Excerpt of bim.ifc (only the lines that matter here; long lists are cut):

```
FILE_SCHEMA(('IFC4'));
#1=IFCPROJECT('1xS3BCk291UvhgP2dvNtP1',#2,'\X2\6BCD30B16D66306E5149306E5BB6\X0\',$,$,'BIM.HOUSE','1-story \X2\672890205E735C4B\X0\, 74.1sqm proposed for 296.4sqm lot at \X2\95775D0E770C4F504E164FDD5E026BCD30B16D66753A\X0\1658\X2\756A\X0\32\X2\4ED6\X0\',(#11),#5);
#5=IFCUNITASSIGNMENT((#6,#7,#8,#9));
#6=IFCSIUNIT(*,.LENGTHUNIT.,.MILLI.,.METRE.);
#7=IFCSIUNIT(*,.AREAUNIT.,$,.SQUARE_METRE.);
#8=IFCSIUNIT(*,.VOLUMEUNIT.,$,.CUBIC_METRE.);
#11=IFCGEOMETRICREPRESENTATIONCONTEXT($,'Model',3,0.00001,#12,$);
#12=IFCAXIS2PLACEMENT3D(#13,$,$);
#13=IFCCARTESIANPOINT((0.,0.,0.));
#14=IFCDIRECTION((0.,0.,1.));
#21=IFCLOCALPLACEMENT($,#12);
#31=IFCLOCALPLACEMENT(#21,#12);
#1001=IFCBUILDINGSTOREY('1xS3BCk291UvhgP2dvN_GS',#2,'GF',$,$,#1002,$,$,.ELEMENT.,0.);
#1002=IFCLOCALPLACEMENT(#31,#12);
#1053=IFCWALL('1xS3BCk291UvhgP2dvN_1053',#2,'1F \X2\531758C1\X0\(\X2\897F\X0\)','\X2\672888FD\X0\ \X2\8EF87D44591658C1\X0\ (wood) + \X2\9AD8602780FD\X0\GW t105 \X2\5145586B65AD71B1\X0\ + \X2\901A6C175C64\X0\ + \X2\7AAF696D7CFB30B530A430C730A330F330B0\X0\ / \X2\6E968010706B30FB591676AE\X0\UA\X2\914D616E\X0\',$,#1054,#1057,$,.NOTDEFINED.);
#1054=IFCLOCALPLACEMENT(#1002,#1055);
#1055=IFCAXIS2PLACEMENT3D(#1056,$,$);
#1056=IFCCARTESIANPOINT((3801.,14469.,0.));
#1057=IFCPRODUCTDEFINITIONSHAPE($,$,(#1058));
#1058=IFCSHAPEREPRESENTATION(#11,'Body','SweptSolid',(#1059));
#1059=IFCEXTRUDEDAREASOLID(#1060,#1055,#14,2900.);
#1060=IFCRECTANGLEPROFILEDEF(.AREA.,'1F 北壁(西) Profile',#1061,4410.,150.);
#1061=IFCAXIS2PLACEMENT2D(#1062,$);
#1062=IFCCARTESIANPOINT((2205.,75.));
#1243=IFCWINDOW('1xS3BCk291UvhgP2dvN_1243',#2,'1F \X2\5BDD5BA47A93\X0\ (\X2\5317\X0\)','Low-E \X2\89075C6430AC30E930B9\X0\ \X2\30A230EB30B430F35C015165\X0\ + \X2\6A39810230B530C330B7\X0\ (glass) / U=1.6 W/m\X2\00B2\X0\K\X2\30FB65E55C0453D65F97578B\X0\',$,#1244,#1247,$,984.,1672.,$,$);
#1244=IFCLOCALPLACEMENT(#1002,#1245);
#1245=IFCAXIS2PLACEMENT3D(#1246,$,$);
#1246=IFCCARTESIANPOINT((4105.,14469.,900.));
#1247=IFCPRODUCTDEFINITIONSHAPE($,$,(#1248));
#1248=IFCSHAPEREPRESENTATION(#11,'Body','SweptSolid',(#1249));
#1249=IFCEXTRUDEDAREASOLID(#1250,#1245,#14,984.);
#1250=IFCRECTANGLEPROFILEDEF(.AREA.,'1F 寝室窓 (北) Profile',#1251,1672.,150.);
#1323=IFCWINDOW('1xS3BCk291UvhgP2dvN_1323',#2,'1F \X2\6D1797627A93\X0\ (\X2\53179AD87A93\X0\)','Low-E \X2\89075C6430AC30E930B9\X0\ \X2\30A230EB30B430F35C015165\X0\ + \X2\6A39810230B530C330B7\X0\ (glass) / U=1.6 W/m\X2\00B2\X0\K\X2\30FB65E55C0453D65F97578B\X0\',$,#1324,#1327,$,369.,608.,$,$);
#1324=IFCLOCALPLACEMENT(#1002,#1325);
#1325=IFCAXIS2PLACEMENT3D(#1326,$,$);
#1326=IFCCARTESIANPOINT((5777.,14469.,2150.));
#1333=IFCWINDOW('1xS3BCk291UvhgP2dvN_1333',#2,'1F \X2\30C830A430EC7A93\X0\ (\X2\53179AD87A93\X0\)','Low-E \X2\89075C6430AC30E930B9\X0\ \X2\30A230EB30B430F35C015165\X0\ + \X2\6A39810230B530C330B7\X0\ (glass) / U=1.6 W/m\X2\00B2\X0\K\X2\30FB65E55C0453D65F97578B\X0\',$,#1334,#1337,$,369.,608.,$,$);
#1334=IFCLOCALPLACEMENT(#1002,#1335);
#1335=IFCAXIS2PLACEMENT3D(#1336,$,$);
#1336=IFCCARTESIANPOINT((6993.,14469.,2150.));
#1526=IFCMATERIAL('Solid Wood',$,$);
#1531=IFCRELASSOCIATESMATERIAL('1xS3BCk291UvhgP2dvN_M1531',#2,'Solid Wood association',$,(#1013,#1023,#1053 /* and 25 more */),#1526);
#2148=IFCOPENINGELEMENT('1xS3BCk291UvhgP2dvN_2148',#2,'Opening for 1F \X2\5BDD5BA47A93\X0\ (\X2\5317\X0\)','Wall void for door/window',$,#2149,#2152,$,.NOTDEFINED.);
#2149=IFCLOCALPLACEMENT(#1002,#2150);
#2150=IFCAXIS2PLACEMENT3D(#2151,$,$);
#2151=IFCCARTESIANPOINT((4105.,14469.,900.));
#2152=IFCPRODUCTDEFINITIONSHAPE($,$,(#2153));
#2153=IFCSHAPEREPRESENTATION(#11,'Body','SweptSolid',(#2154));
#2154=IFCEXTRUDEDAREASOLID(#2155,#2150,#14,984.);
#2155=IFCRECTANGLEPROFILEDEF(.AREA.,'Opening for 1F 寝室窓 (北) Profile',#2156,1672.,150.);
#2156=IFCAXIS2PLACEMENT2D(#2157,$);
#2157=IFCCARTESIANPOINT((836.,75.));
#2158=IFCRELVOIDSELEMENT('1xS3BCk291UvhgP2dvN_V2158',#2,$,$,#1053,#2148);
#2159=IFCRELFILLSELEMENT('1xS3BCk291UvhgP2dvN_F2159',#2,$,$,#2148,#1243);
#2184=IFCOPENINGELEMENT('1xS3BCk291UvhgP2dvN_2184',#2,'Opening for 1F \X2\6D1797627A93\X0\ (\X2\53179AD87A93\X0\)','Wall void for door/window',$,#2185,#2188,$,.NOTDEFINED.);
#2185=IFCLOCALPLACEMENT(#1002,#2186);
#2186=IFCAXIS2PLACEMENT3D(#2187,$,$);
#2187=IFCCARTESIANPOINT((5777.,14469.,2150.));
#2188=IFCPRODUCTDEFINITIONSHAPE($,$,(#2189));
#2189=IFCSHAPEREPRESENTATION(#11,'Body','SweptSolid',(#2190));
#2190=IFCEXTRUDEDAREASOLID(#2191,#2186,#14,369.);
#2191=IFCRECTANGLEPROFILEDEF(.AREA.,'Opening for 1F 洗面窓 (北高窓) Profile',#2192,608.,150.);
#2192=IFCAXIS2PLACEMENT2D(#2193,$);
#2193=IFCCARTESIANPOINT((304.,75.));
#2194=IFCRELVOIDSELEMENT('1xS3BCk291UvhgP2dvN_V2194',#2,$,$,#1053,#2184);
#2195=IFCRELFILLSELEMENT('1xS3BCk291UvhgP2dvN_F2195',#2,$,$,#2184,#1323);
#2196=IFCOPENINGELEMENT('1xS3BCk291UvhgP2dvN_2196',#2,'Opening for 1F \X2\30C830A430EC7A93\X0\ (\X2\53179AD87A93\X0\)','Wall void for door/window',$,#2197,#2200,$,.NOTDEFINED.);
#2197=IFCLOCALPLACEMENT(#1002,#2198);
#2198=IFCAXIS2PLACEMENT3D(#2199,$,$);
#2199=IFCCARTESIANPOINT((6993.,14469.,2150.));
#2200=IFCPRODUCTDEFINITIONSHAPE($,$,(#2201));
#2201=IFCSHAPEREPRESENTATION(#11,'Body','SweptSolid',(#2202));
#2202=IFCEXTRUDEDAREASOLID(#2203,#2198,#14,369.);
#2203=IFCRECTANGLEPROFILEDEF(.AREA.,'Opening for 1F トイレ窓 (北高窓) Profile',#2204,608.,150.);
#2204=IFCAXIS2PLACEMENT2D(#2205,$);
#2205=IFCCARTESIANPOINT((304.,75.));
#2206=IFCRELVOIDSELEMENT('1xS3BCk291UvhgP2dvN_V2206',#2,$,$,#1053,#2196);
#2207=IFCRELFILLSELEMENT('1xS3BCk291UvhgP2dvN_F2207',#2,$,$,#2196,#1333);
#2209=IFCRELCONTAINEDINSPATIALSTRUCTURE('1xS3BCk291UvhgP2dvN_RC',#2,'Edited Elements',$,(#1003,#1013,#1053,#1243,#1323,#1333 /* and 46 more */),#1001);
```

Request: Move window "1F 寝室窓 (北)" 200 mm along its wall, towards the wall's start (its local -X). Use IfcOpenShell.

```python
import ifcopenshell
import ifcopenshell.api.geometry
import ifcopenshell.util.placement
import ifcopenshell.util.unit

model = ifcopenshell.open("bim.ifc")
unit_scale = ifcopenshell.util.unit.calculate_unit_scale(model)

window = model.by_guid("1xS3BCk291UvhgP2dvN_1243")
opening = window.FillsVoids[0].RelatingOpeningElement
wall = opening.VoidsElements[0].RelatingBuildingElement

wall_matrix = ifcopenshell.util.placement.get_local_placement(wall.ObjectPlacement)
shift = wall_matrix[:3, 0] * -0.2 / unit_scale
before = ifcopenshell.util.placement.get_local_placement(window.ObjectPlacement)[:3, 3].copy()

# The window is not placed relative to its opening, so move both.
for product in (opening, window):
    matrix = ifcopenshell.util.placement.get_local_placement(product.ObjectPlacement)
    matrix[:3, 3] += shift
    ifcopenshell.api.geometry.edit_object_placement(model, product=product, matrix=matrix, is_si=False)

after = ifcopenshell.util.placement.get_local_placement(window.ObjectPlacement)[:3, 3]
print("window moved by", (after - before).round(3) + 0.0)

model.write("bim_updated.ifc")
```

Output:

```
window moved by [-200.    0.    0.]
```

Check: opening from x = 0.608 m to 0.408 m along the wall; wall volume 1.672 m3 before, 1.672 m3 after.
